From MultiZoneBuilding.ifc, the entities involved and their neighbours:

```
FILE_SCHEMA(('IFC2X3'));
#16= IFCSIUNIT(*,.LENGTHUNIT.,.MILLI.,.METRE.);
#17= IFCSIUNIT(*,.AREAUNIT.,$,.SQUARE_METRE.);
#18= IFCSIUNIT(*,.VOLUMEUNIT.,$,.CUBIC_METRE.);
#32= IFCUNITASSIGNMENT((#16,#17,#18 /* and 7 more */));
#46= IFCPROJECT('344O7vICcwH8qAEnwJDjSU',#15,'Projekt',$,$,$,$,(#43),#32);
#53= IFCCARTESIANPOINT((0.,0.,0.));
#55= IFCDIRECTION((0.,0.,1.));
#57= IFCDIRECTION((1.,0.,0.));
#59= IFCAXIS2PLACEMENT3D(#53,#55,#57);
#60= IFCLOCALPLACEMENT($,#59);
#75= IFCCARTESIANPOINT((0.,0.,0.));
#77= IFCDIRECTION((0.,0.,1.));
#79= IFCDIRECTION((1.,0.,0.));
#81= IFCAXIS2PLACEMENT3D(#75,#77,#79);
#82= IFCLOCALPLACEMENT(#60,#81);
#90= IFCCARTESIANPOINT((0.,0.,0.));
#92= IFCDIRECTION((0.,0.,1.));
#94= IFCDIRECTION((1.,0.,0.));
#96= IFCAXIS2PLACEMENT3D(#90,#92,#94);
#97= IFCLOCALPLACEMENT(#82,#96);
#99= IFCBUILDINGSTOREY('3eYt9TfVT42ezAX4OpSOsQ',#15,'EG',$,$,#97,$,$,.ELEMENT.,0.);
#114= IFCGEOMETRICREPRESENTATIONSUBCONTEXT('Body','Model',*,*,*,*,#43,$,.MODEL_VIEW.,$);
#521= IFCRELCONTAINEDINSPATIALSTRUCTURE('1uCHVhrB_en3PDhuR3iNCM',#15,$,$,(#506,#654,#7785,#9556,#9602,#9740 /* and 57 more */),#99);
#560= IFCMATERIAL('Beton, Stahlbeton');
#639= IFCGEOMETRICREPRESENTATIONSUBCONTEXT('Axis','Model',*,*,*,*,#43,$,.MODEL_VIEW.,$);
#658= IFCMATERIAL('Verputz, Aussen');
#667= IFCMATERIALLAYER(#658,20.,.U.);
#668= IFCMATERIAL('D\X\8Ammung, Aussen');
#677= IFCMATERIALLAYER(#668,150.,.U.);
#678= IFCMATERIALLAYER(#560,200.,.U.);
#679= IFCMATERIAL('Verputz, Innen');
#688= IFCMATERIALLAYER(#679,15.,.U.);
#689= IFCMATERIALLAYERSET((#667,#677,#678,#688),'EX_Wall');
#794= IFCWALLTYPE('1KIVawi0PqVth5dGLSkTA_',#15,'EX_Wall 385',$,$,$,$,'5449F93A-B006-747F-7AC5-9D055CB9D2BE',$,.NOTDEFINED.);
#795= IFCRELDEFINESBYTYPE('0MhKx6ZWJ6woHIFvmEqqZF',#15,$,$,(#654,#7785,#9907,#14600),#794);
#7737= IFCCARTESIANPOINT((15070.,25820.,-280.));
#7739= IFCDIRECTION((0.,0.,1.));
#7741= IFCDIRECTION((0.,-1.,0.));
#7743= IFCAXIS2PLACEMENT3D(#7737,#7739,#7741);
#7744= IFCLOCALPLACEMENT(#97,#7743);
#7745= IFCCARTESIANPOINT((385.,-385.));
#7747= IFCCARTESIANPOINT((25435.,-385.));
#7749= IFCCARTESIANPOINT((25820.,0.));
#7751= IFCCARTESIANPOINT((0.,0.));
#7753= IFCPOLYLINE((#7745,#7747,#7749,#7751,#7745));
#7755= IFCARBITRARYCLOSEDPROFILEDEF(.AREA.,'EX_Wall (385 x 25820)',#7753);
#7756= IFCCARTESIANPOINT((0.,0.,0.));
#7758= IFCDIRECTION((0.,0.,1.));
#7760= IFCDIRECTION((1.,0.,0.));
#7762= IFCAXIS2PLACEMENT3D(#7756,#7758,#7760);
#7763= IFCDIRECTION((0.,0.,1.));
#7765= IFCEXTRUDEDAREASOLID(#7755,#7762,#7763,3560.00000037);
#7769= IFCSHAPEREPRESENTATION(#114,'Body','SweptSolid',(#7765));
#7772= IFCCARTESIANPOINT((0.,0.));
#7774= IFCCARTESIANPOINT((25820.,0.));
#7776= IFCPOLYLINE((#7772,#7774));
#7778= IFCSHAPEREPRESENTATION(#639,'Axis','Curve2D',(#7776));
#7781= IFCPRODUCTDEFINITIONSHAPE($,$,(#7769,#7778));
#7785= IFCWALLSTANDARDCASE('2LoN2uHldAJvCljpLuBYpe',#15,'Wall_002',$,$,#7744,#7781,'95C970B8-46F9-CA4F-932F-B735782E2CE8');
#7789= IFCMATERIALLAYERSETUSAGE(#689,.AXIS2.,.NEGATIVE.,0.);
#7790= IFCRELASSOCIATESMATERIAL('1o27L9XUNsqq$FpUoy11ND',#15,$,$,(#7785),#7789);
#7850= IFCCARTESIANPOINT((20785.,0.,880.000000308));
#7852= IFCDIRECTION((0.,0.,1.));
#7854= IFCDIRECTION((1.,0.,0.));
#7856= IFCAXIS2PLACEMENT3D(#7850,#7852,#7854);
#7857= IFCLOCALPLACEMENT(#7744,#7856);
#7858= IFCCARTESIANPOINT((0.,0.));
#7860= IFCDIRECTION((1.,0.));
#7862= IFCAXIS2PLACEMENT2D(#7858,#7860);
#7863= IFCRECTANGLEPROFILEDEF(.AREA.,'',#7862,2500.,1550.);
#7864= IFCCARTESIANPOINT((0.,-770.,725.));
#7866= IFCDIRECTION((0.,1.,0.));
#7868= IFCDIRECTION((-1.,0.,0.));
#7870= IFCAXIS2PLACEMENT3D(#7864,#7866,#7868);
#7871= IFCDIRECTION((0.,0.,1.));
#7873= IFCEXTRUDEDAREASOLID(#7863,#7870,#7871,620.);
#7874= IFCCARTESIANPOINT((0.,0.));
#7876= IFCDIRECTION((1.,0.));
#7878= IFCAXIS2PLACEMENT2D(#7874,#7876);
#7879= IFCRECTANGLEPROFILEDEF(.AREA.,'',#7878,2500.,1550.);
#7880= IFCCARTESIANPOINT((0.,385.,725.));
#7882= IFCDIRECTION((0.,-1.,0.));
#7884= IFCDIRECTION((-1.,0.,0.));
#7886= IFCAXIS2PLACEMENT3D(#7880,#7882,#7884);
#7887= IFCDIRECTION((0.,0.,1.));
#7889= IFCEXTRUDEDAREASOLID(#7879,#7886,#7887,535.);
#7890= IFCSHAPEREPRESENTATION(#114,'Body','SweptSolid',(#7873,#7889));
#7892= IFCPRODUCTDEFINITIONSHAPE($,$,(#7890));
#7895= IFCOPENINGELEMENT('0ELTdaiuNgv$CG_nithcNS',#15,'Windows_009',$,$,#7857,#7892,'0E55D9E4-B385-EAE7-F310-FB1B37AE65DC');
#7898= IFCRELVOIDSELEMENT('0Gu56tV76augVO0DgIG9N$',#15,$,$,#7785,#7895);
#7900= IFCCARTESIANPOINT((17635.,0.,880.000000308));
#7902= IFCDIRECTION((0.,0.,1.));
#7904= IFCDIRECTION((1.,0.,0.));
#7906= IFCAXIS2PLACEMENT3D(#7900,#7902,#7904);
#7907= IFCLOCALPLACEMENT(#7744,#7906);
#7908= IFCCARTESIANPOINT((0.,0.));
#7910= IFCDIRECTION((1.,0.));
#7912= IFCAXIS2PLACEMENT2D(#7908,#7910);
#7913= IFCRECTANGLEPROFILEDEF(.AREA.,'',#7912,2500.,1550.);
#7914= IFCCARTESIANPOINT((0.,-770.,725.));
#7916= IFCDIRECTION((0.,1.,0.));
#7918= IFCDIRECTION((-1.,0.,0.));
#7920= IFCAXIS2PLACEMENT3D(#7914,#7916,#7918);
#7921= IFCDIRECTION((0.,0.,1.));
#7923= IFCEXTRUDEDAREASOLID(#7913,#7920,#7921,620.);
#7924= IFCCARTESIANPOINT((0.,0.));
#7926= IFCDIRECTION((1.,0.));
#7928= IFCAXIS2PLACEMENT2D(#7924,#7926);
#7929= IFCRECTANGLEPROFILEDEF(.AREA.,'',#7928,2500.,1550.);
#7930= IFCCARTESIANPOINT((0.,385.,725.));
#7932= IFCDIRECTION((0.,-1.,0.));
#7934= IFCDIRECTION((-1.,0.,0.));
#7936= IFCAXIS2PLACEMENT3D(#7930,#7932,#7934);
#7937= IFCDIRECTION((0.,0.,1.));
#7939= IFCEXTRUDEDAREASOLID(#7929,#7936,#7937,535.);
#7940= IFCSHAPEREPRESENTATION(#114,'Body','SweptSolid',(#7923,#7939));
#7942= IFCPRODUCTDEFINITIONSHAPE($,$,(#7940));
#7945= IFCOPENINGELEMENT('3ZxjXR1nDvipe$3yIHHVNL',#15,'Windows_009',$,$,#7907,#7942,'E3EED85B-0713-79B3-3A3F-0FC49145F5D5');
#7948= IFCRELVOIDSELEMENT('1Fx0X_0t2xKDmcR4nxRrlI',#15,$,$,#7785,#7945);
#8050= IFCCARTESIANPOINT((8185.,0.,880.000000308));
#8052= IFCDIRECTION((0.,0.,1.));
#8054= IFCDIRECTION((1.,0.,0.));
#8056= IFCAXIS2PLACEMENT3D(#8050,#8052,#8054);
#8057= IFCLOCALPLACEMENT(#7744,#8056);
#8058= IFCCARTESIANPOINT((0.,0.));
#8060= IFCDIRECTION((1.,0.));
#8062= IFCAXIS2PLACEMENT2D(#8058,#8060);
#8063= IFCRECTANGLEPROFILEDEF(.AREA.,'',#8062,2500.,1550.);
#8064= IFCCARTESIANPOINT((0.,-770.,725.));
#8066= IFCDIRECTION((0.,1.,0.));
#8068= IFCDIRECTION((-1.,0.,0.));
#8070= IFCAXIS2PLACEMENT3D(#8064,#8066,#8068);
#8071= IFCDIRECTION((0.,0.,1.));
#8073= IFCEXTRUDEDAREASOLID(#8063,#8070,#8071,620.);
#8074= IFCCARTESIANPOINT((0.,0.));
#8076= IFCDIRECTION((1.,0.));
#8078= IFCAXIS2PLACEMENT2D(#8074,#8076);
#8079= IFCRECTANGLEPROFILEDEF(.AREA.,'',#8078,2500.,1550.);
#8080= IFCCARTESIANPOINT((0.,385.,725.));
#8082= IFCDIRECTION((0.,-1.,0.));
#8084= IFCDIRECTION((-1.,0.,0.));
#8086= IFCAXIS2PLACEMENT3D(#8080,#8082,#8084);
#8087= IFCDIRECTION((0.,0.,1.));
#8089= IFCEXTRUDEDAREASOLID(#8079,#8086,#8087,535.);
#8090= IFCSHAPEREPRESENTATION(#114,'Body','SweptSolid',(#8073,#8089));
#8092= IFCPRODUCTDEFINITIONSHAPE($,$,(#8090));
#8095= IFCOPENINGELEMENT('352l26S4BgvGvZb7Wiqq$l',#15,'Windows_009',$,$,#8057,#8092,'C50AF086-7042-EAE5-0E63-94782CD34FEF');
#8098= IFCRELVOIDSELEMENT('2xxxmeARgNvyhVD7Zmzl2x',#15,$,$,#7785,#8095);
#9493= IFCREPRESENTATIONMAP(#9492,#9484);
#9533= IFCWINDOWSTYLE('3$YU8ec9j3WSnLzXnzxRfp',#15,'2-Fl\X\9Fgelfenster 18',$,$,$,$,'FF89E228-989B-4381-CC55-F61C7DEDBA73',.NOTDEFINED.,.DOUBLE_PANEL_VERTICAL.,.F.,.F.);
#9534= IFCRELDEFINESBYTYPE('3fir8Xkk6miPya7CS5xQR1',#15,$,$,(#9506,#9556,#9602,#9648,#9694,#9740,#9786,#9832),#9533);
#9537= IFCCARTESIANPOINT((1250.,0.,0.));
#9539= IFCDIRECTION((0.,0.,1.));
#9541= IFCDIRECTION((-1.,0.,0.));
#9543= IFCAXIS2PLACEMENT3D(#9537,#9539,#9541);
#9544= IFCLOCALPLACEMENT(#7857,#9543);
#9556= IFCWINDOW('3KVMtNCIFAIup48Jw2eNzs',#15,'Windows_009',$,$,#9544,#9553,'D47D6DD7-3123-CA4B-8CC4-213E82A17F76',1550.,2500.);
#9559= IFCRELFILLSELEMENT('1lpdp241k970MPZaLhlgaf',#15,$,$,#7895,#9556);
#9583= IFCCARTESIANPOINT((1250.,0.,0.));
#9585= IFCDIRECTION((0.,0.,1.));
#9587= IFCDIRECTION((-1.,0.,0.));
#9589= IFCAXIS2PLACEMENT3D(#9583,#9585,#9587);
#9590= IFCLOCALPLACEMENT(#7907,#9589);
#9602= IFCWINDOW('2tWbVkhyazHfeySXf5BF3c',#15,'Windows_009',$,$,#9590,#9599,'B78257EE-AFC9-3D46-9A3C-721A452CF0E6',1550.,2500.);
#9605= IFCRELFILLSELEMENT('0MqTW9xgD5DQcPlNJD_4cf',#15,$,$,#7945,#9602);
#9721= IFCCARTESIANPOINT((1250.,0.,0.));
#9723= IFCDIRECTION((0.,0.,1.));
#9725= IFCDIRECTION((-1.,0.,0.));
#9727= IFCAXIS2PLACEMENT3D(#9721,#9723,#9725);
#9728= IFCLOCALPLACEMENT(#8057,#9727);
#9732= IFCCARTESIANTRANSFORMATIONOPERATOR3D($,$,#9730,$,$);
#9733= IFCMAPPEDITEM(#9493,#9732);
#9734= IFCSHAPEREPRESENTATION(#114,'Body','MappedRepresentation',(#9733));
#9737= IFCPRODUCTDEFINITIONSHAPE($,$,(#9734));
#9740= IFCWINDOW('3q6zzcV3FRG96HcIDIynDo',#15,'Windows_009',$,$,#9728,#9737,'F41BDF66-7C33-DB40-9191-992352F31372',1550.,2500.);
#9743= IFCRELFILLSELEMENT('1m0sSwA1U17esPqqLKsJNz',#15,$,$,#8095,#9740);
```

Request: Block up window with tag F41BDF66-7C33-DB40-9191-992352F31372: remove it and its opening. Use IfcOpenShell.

```python
import ifcopenshell
import ifcopenshell.api.feature
import ifcopenshell.api.root
import ifcopenshell.geom
import ifcopenshell.util.shape

model = ifcopenshell.open("MultiZoneBuilding.ifc")
settings = ifcopenshell.geom.settings()


def volume(element):
    """Net volume in cubic metres, openings subtracted."""
    shape = ifcopenshell.geom.create_shape(settings, element)
    return ifcopenshell.util.shape.get_volume(shape.geometry)


window = model.by_guid("3q6zzcV3FRG96HcIDIynDo")
opening = window.FillsVoids[0].RelatingOpeningElement
wall = opening.VoidsElements[0].RelatingBuildingElement
before = volume(wall)

ifcopenshell.api.root.remove_product(model, product=window)
ifcopenshell.api.feature.remove_feature(model, feature=opening)

after = volume(wall)

print(f"wall volume {before:.3f} -> {after:.3f} m3")

model.write("MultiZoneBuilding_v2.ifc")
```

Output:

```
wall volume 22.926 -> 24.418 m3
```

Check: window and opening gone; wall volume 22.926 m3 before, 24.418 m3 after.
